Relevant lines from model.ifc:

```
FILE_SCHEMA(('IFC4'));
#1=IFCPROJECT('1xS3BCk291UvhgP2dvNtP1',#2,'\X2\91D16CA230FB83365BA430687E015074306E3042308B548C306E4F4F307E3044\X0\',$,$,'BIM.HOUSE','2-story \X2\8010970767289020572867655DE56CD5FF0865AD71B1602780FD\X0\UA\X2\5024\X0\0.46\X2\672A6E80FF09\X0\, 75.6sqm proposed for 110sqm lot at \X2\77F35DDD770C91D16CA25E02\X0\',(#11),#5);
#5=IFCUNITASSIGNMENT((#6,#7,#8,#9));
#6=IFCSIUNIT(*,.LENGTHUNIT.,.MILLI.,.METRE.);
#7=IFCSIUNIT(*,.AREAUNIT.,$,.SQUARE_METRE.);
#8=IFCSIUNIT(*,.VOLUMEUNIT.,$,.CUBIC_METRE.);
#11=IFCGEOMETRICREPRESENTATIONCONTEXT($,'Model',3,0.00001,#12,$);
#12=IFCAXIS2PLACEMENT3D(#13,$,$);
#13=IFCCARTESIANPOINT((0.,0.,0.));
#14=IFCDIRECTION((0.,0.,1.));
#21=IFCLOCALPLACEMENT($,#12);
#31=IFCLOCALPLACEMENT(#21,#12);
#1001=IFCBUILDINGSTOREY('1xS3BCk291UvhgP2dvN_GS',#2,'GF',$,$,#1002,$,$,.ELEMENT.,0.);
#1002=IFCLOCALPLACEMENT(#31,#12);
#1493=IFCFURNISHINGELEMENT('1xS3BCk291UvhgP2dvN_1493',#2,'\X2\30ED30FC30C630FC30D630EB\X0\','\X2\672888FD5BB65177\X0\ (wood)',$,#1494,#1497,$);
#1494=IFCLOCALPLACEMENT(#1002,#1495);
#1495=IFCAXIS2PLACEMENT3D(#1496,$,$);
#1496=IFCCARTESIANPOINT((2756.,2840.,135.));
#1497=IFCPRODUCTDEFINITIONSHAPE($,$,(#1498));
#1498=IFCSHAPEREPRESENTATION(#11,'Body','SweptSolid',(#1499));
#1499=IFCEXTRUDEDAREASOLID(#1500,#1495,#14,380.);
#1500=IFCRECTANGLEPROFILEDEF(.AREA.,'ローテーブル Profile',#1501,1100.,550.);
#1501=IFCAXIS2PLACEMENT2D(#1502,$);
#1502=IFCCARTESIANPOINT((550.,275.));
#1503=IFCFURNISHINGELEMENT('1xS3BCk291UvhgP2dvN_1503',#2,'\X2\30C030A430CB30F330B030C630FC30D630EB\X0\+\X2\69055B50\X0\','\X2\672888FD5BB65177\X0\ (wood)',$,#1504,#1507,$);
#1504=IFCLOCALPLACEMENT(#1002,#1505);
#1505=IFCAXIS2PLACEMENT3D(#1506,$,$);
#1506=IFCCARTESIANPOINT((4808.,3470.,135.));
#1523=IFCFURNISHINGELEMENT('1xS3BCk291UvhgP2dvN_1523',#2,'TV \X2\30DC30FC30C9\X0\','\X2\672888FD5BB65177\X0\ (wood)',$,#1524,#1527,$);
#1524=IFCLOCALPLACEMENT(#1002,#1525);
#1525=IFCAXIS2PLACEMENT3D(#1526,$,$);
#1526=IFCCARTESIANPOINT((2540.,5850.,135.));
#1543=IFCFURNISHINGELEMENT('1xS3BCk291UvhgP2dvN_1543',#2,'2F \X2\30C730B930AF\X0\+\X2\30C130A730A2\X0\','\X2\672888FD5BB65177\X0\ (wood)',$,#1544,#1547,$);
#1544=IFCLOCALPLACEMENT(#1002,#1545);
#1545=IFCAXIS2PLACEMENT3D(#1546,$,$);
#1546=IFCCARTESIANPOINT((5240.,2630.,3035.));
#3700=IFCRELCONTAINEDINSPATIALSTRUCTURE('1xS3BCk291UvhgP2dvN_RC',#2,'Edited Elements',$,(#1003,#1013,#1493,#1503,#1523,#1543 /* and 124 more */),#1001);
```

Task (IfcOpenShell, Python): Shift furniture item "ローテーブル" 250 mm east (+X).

```python
import ifcopenshell
import ifcopenshell.api.geometry
import ifcopenshell.util.placement
import ifcopenshell.util.unit

model = ifcopenshell.open("model.ifc")
unit_scale = ifcopenshell.util.unit.calculate_unit_scale(model)

item = model.by_id(1493)
matrix = ifcopenshell.util.placement.get_local_placement(item.ObjectPlacement)
matrix[0, 3] += 0.25 / unit_scale
ifcopenshell.api.geometry.edit_object_placement(model, product=item, matrix=matrix, is_si=False)

print(ifcopenshell.util.placement.get_local_placement(item.ObjectPlacement).round(3) + 0.0)

model.write("model-out.ifc")
```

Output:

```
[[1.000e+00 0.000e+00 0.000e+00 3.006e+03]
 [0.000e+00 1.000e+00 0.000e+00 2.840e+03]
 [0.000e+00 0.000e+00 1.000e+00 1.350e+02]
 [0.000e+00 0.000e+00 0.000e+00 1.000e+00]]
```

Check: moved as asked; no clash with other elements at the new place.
